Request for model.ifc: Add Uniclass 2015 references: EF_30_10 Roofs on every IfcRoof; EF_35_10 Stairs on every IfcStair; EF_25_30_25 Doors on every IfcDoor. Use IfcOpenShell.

First a look at what the model holds.

```python
import ifcopenshell

model = ifcopenshell.open("model.ifc")
print(model.schema)
print("classifications:", [c.Name for c in model.by_type("IfcClassification")])
for ifc_class in ("IfcDoor", "IfcRoof", "IfcStair", "IfcWall", "IfcWindow"):
    print(ifc_class, len(model.by_type(ifc_class)))
```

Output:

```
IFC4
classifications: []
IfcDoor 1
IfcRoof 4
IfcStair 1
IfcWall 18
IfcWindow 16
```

```python
import ifcopenshell
import ifcopenshell.api.classification

model = ifcopenshell.open("model.ifc")

system = ifcopenshell.api.classification.add_classification(model, classification="Uniclass 2015")

codes = {
    "IfcRoof": ("EF_30_10", "Roofs"),
    "IfcStair": ("EF_35_10", "Stairs"),
    "IfcDoor": ("EF_25_30_25", "Doors"),
}
for ifc_class, (code, name) in codes.items():
    products = model.by_type(ifc_class)
    ifcopenshell.api.classification.add_reference(
        model, products=products, classification=system, identification=code, name=name
    )
    print(code, len(products))

model.write("model_v2.ifc")
```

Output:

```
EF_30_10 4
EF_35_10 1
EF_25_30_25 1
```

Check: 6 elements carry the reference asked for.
